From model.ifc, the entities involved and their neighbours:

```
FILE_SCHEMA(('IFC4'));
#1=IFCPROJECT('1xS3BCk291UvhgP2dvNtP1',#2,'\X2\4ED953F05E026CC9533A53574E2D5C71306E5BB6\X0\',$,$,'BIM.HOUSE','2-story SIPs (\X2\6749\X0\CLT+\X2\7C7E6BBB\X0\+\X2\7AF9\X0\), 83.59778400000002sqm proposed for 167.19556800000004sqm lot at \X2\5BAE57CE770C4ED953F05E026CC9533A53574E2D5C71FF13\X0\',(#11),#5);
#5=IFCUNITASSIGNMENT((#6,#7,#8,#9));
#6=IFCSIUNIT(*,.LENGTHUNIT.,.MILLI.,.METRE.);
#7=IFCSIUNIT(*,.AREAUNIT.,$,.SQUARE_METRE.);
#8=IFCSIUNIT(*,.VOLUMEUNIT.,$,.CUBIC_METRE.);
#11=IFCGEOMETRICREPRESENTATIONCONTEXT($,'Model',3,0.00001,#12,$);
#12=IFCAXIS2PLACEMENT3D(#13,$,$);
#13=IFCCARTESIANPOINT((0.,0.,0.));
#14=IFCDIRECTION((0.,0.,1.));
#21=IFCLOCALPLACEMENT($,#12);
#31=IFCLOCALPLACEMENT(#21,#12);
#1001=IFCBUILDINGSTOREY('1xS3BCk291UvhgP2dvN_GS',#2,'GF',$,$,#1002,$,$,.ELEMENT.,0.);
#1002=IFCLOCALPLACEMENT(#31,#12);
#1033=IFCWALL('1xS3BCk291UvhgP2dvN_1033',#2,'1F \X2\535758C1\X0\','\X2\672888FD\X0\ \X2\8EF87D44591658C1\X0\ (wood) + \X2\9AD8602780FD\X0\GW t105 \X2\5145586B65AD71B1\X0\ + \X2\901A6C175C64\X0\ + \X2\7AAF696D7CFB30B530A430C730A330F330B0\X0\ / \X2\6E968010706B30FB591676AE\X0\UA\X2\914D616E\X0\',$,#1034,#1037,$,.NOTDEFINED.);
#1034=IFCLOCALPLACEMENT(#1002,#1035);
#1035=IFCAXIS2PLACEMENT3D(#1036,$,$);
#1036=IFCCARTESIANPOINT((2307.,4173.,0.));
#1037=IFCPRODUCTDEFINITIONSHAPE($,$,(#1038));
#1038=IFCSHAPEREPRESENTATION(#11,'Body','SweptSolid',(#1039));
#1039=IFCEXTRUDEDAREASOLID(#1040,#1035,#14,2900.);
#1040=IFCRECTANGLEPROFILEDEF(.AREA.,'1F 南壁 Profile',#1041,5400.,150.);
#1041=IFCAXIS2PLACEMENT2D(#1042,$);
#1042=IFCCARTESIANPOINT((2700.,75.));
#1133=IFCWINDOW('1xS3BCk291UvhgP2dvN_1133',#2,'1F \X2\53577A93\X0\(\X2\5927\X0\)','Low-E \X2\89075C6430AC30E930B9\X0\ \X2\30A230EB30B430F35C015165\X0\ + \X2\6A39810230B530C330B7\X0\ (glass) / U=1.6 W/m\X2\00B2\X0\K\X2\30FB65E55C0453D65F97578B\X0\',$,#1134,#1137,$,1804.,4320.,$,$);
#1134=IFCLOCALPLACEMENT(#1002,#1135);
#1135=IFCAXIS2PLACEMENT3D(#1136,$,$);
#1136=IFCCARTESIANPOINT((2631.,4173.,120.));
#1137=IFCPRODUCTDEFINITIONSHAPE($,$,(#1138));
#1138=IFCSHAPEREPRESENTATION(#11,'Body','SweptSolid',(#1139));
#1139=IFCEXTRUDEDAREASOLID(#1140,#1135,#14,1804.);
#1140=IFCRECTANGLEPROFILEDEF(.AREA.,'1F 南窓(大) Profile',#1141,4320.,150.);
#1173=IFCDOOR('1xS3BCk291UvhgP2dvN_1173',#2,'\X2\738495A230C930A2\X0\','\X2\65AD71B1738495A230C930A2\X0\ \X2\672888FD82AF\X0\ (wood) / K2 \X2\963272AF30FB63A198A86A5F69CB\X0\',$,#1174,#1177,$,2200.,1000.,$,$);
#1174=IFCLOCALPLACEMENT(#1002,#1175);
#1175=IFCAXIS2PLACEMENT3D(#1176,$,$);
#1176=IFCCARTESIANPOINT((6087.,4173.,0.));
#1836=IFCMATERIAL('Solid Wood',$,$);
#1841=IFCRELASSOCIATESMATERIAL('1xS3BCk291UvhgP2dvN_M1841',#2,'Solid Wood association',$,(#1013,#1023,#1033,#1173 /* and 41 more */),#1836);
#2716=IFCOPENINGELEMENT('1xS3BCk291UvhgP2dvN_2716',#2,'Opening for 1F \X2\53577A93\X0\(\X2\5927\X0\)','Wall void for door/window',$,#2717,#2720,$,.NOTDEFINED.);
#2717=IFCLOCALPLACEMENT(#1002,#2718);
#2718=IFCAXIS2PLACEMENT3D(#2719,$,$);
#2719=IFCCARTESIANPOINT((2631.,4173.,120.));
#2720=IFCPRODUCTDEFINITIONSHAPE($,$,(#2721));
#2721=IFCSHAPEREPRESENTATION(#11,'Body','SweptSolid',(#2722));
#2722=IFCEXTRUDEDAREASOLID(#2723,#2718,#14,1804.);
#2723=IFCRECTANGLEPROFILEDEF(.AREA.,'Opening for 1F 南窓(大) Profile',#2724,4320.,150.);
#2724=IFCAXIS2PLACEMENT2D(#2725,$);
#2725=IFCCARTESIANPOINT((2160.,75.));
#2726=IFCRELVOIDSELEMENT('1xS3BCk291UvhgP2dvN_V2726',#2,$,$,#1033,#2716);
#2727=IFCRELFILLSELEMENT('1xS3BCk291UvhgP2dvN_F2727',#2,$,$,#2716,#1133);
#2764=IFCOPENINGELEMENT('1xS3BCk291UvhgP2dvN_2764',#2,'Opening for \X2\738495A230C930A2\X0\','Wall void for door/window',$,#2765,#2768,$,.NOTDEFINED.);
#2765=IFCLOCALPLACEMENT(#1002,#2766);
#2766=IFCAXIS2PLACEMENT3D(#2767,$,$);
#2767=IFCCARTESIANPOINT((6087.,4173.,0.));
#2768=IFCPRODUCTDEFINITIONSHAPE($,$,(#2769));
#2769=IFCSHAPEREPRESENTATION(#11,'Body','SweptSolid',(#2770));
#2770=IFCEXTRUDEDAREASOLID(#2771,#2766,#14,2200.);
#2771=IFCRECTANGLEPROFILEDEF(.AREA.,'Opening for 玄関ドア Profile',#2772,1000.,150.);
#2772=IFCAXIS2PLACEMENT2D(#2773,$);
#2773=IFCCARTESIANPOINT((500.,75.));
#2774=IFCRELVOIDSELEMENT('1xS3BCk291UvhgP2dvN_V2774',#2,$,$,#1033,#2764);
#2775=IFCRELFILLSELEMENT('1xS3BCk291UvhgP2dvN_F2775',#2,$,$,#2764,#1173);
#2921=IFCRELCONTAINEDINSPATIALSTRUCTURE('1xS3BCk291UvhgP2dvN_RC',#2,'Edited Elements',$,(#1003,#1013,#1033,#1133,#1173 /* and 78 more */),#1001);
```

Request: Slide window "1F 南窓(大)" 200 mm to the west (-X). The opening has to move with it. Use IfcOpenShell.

```python
import ifcopenshell
import ifcopenshell.api.geometry
import ifcopenshell.util.placement
import ifcopenshell.util.unit

model = ifcopenshell.open("model.ifc")
unit_scale = ifcopenshell.util.unit.calculate_unit_scale(model)

window = model.by_guid("1xS3BCk291UvhgP2dvN_1133")
opening = window.FillsVoids[0].RelatingOpeningElement
wall = opening.VoidsElements[0].RelatingBuildingElement

wall_matrix = ifcopenshell.util.placement.get_local_placement(wall.ObjectPlacement)
shift = wall_matrix[:3, 0] * -0.2 / unit_scale
before = ifcopenshell.util.placement.get_local_placement(window.ObjectPlacement)[:3, 3].copy()

# The window is not placed relative to its opening, so move both.
for product in (opening, window):
    matrix = ifcopenshell.util.placement.get_local_placement(product.ObjectPlacement)
    matrix[:3, 3] += shift
    ifcopenshell.api.geometry.edit_object_placement(model, product=product, matrix=matrix, is_si=False)

after = ifcopenshell.util.placement.get_local_placement(window.ObjectPlacement)[:3, 3]
print("window moved by", (after - before).round(3) + 0.0)

model.write("model_rev.ifc")
```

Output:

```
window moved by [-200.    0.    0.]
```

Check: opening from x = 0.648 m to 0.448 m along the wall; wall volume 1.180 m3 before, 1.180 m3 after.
